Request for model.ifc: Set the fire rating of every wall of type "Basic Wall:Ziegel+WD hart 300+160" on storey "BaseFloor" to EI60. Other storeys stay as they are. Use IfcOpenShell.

First a look at what the model holds.

```python
import ifcopenshell
import ifcopenshell.util.element

model = ifcopenshell.open("model.ifc")
print(model.schema)
storey = next(s for s in model.by_type("IfcBuildingStorey") if s.Name == "BaseFloor")
walls = [e for e in ifcopenshell.util.element.get_decomposition(storey) if e.is_a("IfcWall")]
seen = {}
for e in walls:
    element_type = ifcopenshell.util.element.get_type(e)
    key = (element_type.Name if element_type != e and element_type else None, ifcopenshell.util.element.get_pset(e, "Pset_WallCommon", "FireRating"))
    seen[key] = seen.get(key, 0) + 1
for (name, value), count in sorted(seen.items(), key=str):
    print(count, "x", name, "|", value)
```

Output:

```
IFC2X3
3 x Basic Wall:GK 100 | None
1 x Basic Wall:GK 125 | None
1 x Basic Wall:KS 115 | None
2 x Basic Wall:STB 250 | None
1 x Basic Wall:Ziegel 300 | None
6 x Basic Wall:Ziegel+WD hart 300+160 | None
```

```python
import ifcopenshell
import ifcopenshell.api.pset
import ifcopenshell.util.element

model = ifcopenshell.open("model.ifc")

storey = next(s for s in model.by_type("IfcBuildingStorey") if s.Name == "BaseFloor")
walls = [e for e in ifcopenshell.util.element.get_decomposition(storey) if e.is_a("IfcWall")]

count = 0
for e in walls:
    element_type = ifcopenshell.util.element.get_type(e)
    if element_type in (None, e) or element_type.Name != "Basic Wall:Ziegel+WD hart 300+160":
        continue
    # add_pset returns the element's existing set when there is one.
    pset = ifcopenshell.api.pset.add_pset(model, product=e, name="Pset_WallCommon")
    ifcopenshell.api.pset.edit_pset(model, pset=pset, properties={"FireRating": "EI60"})
    count += 1

print(count, "walls updated")

model.write("model_updated.ifc")
```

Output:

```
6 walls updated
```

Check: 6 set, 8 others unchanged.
